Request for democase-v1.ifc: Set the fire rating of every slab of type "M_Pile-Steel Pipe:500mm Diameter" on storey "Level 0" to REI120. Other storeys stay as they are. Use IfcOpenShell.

First a look at what the model holds.

```python
import ifcopenshell
import ifcopenshell.util.element

model = ifcopenshell.open("democase-v1.ifc")
print(model.schema)
storey = next(s for s in model.by_type("IfcBuildingStorey") if s.Name == "Level 0")
slabs = [e for e in ifcopenshell.util.element.get_decomposition(storey) if e.is_a("IfcSlab")]
seen = {}
for e in slabs:
    element_type = ifcopenshell.util.element.get_type(e)
    key = (element_type.Name if element_type != e and element_type else None, ifcopenshell.util.element.get_pset(e, "Pset_SlabCommon", "FireRating"))
    seen[key] = seen.get(key, 0) + 1
for (name, value), count in sorted(seen.items(), key=str):
    print(count, "x", name, "|", value)
```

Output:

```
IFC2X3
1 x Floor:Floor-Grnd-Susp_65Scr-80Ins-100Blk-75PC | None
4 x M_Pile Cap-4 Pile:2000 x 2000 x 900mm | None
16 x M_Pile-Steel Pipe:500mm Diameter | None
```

```python
import ifcopenshell
import ifcopenshell.api.pset
import ifcopenshell.util.element

model = ifcopenshell.open("democase-v1.ifc")

storey = next(s for s in model.by_type("IfcBuildingStorey") if s.Name == "Level 0")
slabs = [e for e in ifcopenshell.util.element.get_decomposition(storey) if e.is_a("IfcSlab")]

count = 0
for e in slabs:
    element_type = ifcopenshell.util.element.get_type(e)
    if element_type in (None, e) or element_type.Name != "M_Pile-Steel Pipe:500mm Diameter":
        continue
    # add_pset returns the element's existing set when there is one.
    pset = ifcopenshell.api.pset.add_pset(model, product=e, name="Pset_SlabCommon")
    ifcopenshell.api.pset.edit_pset(model, pset=pset, properties={"FireRating": "REI120"})
    count += 1

print(count, "slabs updated")

model.write("democase-v1_updated.ifc")
```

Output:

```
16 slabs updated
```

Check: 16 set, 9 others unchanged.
